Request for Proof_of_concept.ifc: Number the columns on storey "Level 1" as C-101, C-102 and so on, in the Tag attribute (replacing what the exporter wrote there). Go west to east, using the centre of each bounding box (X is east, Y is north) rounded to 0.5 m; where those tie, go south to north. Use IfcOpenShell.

First a look at what the model holds.

```python
import ifcopenshell
import ifcopenshell.util.element
import ifcopenshell.util.placement

model = ifcopenshell.open("Proof_of_concept.ifc")
print(model.schema)
storey = next(s for s in model.by_type("IfcBuildingStorey") if s.Name == "Level 1")
columns = [e for e in ifcopenshell.util.element.get_decomposition(storey) if e.is_a("IfcColumn")]
for e in sorted(columns, key=lambda e: e.id()):
    origin = ifcopenshell.util.placement.get_local_placement(e.ObjectPlacement)[:3, 3]
    print(e.id(), e.Tag, e.Name, origin.round(2) + 0.0, sep=" | ")
```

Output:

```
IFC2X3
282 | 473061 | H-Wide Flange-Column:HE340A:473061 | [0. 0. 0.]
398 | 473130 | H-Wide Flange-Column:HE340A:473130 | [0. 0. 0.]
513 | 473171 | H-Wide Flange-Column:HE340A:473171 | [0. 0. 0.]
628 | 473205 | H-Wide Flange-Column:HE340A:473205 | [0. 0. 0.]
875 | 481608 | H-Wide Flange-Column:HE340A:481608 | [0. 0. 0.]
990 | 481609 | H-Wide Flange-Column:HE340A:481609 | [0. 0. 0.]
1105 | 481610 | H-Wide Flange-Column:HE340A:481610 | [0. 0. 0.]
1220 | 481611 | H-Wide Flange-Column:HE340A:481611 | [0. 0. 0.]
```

```python
import ifcopenshell
import ifcopenshell.geom
import ifcopenshell.util.element
import ifcopenshell.util.shape

model = ifcopenshell.open("Proof_of_concept.ifc")
settings = ifcopenshell.geom.settings()
settings.set("use-world-coords", True)


def centre(element):
    shape = ifcopenshell.geom.create_shape(settings, element)
    return ifcopenshell.util.shape.get_bbox_centroid(shape.geometry)


storey = next(s for s in model.by_type("IfcBuildingStorey") if s.Name == "Level 1")
columns = [e for e in ifcopenshell.util.element.get_decomposition(storey) if e.is_a("IfcColumn")]

# Insertion points can sit at a corner or the storey origin, so sort by the geometry (in metres).
centres = {e: centre(e) for e in columns}
columns.sort(key=lambda e: (round(centres[e][0] / 0.5), centres[e][1]))

for i, e in enumerate(columns, start=1):
    number = f"C-1{i:02d}"
    e.Tag = number
    print(e.id(), number)

model.write("Proof_of_concept_rev.ifc")
```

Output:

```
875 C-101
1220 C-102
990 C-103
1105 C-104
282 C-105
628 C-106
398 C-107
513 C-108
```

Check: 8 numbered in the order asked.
